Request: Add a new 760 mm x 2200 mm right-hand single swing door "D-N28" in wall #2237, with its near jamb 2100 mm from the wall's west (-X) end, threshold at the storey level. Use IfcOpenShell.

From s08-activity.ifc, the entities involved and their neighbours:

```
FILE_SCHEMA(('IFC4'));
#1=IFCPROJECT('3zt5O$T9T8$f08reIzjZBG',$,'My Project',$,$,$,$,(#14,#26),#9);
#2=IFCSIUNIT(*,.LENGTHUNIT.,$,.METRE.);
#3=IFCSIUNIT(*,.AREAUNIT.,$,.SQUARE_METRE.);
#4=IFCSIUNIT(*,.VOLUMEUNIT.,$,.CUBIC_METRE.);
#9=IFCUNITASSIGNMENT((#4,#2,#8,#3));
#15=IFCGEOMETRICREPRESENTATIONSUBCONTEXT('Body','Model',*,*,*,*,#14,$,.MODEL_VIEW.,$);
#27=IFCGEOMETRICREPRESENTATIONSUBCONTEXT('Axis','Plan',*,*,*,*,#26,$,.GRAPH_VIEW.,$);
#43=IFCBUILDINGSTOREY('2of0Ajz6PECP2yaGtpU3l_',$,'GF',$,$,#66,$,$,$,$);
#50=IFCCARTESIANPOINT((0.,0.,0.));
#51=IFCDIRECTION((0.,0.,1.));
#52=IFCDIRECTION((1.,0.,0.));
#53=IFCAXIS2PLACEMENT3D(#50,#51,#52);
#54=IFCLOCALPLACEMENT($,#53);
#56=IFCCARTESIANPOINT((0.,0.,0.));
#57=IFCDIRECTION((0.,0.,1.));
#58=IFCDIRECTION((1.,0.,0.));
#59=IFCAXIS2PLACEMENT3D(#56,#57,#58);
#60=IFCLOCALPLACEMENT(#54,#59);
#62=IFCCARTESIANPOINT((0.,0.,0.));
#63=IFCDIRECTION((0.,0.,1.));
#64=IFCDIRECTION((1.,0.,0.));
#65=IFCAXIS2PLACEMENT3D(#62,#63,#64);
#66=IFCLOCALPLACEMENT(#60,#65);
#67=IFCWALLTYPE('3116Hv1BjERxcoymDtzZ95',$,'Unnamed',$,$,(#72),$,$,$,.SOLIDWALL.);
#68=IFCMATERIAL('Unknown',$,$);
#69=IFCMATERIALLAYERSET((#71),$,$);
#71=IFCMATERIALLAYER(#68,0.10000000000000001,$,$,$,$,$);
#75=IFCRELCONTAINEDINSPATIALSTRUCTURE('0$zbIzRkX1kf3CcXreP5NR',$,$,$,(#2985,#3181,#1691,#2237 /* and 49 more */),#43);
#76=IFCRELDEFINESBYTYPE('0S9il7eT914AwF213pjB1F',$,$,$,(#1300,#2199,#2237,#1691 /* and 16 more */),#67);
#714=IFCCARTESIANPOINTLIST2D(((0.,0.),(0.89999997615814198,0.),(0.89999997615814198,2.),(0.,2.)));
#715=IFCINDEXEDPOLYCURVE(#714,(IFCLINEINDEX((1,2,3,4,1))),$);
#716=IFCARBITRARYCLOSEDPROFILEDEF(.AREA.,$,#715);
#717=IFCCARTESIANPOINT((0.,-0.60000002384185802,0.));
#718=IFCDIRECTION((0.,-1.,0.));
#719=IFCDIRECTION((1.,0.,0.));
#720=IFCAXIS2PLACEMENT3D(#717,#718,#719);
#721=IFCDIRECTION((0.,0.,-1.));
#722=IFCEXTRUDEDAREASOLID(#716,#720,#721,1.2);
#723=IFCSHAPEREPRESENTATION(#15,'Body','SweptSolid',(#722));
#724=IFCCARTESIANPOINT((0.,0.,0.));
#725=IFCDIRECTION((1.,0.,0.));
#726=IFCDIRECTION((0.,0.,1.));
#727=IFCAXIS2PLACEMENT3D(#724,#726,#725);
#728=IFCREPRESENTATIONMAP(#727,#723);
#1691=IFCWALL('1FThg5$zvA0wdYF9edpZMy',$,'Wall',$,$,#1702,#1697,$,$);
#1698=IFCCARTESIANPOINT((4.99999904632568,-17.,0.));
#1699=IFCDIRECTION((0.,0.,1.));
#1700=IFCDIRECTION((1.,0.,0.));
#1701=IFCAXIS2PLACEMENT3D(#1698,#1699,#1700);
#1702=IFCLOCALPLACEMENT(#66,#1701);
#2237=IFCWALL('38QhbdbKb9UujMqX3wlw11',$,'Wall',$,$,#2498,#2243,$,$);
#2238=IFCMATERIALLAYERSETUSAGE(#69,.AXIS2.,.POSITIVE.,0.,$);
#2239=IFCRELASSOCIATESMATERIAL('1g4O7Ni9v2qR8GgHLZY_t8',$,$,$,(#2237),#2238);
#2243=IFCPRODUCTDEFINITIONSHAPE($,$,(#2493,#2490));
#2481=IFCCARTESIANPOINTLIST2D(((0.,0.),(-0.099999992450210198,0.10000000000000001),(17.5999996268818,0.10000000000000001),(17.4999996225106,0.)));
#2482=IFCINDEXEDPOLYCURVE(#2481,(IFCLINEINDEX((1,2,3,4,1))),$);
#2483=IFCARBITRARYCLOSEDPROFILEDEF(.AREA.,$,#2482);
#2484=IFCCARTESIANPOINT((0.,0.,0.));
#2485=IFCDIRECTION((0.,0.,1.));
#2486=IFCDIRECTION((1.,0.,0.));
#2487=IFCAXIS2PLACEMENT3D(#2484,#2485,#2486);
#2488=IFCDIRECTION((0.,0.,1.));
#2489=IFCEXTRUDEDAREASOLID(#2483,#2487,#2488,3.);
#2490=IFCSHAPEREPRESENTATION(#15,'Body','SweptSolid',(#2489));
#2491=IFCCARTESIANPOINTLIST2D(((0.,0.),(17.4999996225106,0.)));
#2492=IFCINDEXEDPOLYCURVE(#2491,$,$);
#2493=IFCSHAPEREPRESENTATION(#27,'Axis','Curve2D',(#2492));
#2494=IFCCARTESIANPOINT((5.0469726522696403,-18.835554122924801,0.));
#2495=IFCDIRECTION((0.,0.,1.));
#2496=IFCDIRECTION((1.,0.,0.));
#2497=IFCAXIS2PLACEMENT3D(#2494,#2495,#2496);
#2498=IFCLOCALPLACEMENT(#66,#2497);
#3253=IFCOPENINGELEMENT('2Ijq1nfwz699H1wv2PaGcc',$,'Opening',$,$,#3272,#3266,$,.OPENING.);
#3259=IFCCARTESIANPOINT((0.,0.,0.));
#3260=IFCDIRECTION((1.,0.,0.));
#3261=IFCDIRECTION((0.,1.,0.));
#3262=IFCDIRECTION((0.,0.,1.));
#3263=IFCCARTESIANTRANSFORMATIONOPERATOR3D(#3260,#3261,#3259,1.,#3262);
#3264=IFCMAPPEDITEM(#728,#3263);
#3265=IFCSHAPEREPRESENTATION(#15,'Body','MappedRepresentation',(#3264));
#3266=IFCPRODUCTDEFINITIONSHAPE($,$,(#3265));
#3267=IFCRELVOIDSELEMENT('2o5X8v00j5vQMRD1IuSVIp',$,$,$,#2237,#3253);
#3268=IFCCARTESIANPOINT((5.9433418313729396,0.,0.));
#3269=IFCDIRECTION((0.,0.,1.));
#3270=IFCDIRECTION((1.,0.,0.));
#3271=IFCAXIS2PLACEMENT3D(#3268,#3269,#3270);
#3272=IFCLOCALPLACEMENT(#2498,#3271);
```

```python
import numpy as np
import ifcopenshell
import ifcopenshell.api.feature
import ifcopenshell.api.geometry
import ifcopenshell.api.root
import ifcopenshell.api.spatial
import ifcopenshell.geom
import ifcopenshell.util.element
import ifcopenshell.util.placement
import ifcopenshell.util.representation
import ifcopenshell.util.shape
import ifcopenshell.util.unit

model = ifcopenshell.open("s08-activity.ifc")
unit_scale = ifcopenshell.util.unit.calculate_unit_scale(model)
settings = ifcopenshell.geom.settings()


def volume(element):
    """Net volume in cubic metres, openings subtracted."""
    shape = ifcopenshell.geom.create_shape(settings, element)
    return ifcopenshell.util.shape.get_volume(shape.geometry)


wall = model.by_guid("38QhbdbKb9UujMqX3wlw11")
storey = ifcopenshell.util.element.get_container(wall, ifc_class="IfcBuildingStorey")
context = ifcopenshell.util.representation.get_context(model, "Model", "Body", "MODEL_VIEW")
before = volume(wall)

width, height, from_end, sill = 0.76, 2.2, 2.1, 0.0  # metres

# The wall runs along its own X axis, and the end named is its -X end.
wall_shape = ifcopenshell.geom.create_shape(settings, wall)
x, y, z = ifcopenshell.util.shape.get_vertices(wall_shape.geometry).T
start = x.min() + from_end
face, thickness = float(y.min()), float(y.max() - y.min())
wall_matrix = ifcopenshell.util.placement.get_local_placement(wall.ObjectPlacement)
level = ifcopenshell.util.placement.get_local_placement(storey.ObjectPlacement)[2, 3]


def in_wall(x, y):
    """Placement at x, y metres in the wall's axes, at sill height."""
    matrix = wall_matrix.copy()
    matrix[:, 3] = wall_matrix @ np.array([x / unit_scale, y / unit_scale, 0.0, 1.0])
    matrix[2, 3] = level + sill / unit_scale
    return matrix


# Opening: a box that overshoots both wall faces by 50 mm.
opening = ifcopenshell.api.root.create_entity(model, ifc_class="IfcOpeningElement", predefined_type="OPENING")
box = ifcopenshell.api.geometry.add_wall_representation(
    model, context=context, length=width, height=height, thickness=thickness + 0.1
)
ifcopenshell.api.geometry.assign_representation(model, product=opening, representation=box)
ifcopenshell.api.geometry.edit_object_placement(model, product=opening, matrix=in_wall(start, face - 0.05), is_si=False)
ifcopenshell.api.feature.add_feature(model, feature=opening, element=wall)

door = ifcopenshell.api.root.create_entity(model, ifc_class="IfcDoor", name="D-N28", predefined_type="DOOR")
door.OverallWidth, door.OverallHeight = width / unit_scale, height / unit_scale
door.OperationType = "SINGLE_SWING_RIGHT"
body = ifcopenshell.api.geometry.add_door_representation(
    model,
    context=context,
    overall_width=door.OverallWidth,
    overall_height=door.OverallHeight,
    operation_type="SINGLE_SWING_RIGHT",
    lining_properties={"LiningDepth": thickness / unit_scale, "ThresholdDepth": thickness / unit_scale},
)
ifcopenshell.api.geometry.assign_representation(model, product=door, representation=body)
ifcopenshell.api.spatial.assign_container(model, products=[door], relating_structure=storey)
ifcopenshell.api.feature.add_filling(model, opening=opening, element=door)

# The lining spans the wall, so the door starts at the wall face.
ifcopenshell.api.geometry.edit_object_placement(model, product=door, matrix=in_wall(start, face), is_si=False)

after = volume(wall)

print(f"wall volume {before:.3f} -> {after:.3f} m3")

model.write("s08-activity_v2.ifc")
```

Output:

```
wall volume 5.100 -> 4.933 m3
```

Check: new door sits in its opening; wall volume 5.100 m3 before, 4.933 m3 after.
